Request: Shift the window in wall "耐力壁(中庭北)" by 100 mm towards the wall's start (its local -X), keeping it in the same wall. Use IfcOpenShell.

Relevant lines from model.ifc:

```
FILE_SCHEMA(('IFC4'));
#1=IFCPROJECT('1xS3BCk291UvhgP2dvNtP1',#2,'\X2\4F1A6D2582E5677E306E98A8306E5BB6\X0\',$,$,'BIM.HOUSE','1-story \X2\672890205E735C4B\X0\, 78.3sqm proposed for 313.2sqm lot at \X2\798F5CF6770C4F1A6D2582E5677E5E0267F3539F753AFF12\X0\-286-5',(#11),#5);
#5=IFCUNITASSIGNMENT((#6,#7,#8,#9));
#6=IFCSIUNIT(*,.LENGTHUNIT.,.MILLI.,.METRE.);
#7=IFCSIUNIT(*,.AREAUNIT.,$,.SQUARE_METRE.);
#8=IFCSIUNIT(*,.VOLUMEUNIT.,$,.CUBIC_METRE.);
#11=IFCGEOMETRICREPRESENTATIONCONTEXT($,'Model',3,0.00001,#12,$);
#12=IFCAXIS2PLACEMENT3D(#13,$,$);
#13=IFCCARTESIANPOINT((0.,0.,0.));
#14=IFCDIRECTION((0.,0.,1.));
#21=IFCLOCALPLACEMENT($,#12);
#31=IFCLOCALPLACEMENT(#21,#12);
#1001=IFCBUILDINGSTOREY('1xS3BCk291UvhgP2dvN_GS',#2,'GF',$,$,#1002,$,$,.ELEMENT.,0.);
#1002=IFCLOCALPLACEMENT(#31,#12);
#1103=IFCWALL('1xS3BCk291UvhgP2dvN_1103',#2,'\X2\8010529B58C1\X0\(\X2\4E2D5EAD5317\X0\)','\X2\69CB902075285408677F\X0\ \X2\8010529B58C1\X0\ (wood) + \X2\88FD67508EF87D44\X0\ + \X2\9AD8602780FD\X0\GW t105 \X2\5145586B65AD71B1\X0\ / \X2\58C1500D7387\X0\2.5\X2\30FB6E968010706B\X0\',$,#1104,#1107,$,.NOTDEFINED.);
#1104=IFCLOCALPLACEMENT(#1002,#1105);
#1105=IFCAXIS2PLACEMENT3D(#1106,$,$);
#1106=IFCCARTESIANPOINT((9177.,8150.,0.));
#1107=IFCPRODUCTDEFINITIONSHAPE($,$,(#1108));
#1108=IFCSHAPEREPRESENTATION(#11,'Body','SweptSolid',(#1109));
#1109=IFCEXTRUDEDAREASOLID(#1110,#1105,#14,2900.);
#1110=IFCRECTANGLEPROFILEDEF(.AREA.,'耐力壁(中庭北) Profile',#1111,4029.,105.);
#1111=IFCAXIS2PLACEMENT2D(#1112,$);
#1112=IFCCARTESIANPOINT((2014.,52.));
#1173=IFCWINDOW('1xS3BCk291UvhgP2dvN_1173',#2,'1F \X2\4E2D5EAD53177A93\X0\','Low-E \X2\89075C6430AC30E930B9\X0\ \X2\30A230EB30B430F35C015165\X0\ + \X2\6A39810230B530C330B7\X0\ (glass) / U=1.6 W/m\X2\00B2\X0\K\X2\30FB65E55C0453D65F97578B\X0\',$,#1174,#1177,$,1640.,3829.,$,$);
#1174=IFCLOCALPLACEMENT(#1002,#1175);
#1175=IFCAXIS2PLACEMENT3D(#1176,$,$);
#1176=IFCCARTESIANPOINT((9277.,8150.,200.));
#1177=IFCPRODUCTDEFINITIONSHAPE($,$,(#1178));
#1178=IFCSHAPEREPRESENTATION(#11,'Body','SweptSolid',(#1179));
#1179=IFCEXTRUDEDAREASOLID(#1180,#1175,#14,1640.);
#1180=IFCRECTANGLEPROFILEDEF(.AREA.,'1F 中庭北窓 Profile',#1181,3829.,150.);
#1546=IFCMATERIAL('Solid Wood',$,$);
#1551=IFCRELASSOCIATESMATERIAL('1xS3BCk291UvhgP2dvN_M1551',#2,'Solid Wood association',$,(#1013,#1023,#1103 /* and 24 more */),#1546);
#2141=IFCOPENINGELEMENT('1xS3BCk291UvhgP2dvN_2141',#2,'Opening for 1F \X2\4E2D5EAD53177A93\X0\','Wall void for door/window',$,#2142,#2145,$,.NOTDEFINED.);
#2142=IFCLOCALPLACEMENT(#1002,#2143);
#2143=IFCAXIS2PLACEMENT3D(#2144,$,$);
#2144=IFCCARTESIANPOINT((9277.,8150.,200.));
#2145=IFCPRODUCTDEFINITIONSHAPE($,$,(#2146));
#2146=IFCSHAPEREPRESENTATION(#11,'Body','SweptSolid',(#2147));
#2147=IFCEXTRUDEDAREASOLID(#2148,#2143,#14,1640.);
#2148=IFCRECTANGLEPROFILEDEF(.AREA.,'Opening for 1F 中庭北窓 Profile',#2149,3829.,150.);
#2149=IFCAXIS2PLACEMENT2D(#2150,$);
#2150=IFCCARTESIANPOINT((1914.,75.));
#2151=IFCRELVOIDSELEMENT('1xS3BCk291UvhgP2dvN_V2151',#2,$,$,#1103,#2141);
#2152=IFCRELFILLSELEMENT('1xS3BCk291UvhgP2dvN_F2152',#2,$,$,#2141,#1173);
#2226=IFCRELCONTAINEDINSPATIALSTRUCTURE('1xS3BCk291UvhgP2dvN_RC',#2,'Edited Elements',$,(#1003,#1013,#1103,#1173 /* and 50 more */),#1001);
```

```python
import ifcopenshell
import ifcopenshell.api.geometry
import ifcopenshell.util.placement
import ifcopenshell.util.unit

model = ifcopenshell.open("model.ifc")
unit_scale = ifcopenshell.util.unit.calculate_unit_scale(model)

window = model.by_id(1173)
opening = window.FillsVoids[0].RelatingOpeningElement
wall = opening.VoidsElements[0].RelatingBuildingElement

wall_matrix = ifcopenshell.util.placement.get_local_placement(wall.ObjectPlacement)
shift = wall_matrix[:3, 0] * -0.1 / unit_scale
before = ifcopenshell.util.placement.get_local_placement(window.ObjectPlacement)[:3, 3].copy()

# The window is not placed relative to its opening, so move both.
for product in (opening, window):
    matrix = ifcopenshell.util.placement.get_local_placement(product.ObjectPlacement)
    matrix[:3, 3] += shift
    ifcopenshell.api.geometry.edit_object_placement(model, product=product, matrix=matrix, is_si=False)

after = ifcopenshell.util.placement.get_local_placement(window.ObjectPlacement)[:3, 3]
print("window moved by", (after - before).round(3) + 0.0)

model.write("model-out.ifc")
```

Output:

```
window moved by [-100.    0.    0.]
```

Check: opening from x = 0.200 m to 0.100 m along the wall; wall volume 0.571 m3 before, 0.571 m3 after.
